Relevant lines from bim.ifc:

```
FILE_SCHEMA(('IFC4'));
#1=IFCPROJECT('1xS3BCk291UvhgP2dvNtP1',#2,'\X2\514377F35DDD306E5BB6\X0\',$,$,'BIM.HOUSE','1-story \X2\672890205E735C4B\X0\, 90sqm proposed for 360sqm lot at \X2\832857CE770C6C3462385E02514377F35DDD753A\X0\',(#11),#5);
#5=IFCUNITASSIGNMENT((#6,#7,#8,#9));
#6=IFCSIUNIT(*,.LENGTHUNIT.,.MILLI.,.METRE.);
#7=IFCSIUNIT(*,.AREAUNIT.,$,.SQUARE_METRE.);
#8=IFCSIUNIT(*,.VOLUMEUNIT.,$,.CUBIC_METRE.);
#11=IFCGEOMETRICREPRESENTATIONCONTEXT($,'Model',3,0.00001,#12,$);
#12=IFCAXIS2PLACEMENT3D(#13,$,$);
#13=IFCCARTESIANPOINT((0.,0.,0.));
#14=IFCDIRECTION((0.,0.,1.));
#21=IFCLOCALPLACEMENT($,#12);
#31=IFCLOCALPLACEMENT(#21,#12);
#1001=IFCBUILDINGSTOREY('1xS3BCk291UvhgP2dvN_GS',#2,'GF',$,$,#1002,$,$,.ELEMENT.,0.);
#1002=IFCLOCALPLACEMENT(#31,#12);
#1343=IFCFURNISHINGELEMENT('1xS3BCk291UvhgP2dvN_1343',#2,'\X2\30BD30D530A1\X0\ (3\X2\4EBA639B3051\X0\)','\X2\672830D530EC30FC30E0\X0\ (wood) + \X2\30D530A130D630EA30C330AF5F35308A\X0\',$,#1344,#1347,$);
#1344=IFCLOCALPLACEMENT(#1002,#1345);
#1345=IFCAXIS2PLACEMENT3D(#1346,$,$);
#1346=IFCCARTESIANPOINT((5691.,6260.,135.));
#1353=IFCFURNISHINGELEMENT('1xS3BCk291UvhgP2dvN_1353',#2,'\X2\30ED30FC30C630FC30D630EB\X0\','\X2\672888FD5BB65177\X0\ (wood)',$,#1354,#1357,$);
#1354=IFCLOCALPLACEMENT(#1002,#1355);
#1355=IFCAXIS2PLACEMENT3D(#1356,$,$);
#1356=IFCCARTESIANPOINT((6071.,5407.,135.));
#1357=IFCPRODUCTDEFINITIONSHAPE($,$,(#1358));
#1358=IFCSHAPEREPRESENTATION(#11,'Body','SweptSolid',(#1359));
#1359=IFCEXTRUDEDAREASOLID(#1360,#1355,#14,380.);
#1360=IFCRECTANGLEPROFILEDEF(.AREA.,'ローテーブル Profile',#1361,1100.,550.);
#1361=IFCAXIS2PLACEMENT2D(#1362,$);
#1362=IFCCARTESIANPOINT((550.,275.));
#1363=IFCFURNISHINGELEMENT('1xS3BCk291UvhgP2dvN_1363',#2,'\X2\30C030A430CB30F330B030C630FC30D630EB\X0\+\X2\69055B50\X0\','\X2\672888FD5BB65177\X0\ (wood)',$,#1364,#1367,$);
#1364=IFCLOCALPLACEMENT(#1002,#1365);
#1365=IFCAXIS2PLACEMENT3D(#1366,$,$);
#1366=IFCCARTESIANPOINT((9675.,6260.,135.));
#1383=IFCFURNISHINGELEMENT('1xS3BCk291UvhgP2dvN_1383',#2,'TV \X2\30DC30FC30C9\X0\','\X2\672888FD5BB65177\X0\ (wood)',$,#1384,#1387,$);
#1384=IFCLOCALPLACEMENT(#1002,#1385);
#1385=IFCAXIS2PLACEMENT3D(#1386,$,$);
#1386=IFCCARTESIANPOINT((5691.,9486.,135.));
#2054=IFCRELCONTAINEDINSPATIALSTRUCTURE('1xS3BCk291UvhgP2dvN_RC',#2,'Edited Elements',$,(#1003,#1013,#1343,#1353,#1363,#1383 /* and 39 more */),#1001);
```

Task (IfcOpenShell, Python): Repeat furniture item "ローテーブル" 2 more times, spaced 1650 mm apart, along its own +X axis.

```python
import ifcopenshell
import ifcopenshell.api.geometry
import ifcopenshell.api.root
import ifcopenshell.util.element
import ifcopenshell.util.placement

model = ifcopenshell.open("bim.ifc")


def reuse_history(source, copy):
    """copy_class also copies each property set's owner history, people and application; keep the originals."""
    for rel in copy.IsDefinedBy:
        if rel.is_a("IfcRelDefinesByProperties") and (history := rel.RelatingPropertyDefinition.OwnerHistory):
            rel.RelatingPropertyDefinition.OwnerHistory = source.OwnerHistory
            ifcopenshell.util.element.remove_deep2(model, history)


source = model.by_guid("1xS3BCk291UvhgP2dvN_1353")
base = ifcopenshell.util.placement.get_local_placement(source.ObjectPlacement)
step = base[:3, 0] * 1650.0

for i in range(1, 3):
    copy = ifcopenshell.api.root.copy_class(model, product=source)
    copy.Representation = ifcopenshell.util.element.copy_deep(
        model, source.Representation, exclude=["IfcGeometricRepresentationContext", "IfcRepresentationMap"]
    )
    reuse_history(source, copy)
    matrix = base.copy()
    matrix[:3, 3] += i * step
    print("added at", matrix[:3, 3].round(3) + 0.0)
    ifcopenshell.api.geometry.edit_object_placement(model, product=copy, matrix=matrix, is_si=False)

model.write("bim_edited.ifc")
```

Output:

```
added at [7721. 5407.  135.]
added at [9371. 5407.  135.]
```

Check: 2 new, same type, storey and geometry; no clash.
